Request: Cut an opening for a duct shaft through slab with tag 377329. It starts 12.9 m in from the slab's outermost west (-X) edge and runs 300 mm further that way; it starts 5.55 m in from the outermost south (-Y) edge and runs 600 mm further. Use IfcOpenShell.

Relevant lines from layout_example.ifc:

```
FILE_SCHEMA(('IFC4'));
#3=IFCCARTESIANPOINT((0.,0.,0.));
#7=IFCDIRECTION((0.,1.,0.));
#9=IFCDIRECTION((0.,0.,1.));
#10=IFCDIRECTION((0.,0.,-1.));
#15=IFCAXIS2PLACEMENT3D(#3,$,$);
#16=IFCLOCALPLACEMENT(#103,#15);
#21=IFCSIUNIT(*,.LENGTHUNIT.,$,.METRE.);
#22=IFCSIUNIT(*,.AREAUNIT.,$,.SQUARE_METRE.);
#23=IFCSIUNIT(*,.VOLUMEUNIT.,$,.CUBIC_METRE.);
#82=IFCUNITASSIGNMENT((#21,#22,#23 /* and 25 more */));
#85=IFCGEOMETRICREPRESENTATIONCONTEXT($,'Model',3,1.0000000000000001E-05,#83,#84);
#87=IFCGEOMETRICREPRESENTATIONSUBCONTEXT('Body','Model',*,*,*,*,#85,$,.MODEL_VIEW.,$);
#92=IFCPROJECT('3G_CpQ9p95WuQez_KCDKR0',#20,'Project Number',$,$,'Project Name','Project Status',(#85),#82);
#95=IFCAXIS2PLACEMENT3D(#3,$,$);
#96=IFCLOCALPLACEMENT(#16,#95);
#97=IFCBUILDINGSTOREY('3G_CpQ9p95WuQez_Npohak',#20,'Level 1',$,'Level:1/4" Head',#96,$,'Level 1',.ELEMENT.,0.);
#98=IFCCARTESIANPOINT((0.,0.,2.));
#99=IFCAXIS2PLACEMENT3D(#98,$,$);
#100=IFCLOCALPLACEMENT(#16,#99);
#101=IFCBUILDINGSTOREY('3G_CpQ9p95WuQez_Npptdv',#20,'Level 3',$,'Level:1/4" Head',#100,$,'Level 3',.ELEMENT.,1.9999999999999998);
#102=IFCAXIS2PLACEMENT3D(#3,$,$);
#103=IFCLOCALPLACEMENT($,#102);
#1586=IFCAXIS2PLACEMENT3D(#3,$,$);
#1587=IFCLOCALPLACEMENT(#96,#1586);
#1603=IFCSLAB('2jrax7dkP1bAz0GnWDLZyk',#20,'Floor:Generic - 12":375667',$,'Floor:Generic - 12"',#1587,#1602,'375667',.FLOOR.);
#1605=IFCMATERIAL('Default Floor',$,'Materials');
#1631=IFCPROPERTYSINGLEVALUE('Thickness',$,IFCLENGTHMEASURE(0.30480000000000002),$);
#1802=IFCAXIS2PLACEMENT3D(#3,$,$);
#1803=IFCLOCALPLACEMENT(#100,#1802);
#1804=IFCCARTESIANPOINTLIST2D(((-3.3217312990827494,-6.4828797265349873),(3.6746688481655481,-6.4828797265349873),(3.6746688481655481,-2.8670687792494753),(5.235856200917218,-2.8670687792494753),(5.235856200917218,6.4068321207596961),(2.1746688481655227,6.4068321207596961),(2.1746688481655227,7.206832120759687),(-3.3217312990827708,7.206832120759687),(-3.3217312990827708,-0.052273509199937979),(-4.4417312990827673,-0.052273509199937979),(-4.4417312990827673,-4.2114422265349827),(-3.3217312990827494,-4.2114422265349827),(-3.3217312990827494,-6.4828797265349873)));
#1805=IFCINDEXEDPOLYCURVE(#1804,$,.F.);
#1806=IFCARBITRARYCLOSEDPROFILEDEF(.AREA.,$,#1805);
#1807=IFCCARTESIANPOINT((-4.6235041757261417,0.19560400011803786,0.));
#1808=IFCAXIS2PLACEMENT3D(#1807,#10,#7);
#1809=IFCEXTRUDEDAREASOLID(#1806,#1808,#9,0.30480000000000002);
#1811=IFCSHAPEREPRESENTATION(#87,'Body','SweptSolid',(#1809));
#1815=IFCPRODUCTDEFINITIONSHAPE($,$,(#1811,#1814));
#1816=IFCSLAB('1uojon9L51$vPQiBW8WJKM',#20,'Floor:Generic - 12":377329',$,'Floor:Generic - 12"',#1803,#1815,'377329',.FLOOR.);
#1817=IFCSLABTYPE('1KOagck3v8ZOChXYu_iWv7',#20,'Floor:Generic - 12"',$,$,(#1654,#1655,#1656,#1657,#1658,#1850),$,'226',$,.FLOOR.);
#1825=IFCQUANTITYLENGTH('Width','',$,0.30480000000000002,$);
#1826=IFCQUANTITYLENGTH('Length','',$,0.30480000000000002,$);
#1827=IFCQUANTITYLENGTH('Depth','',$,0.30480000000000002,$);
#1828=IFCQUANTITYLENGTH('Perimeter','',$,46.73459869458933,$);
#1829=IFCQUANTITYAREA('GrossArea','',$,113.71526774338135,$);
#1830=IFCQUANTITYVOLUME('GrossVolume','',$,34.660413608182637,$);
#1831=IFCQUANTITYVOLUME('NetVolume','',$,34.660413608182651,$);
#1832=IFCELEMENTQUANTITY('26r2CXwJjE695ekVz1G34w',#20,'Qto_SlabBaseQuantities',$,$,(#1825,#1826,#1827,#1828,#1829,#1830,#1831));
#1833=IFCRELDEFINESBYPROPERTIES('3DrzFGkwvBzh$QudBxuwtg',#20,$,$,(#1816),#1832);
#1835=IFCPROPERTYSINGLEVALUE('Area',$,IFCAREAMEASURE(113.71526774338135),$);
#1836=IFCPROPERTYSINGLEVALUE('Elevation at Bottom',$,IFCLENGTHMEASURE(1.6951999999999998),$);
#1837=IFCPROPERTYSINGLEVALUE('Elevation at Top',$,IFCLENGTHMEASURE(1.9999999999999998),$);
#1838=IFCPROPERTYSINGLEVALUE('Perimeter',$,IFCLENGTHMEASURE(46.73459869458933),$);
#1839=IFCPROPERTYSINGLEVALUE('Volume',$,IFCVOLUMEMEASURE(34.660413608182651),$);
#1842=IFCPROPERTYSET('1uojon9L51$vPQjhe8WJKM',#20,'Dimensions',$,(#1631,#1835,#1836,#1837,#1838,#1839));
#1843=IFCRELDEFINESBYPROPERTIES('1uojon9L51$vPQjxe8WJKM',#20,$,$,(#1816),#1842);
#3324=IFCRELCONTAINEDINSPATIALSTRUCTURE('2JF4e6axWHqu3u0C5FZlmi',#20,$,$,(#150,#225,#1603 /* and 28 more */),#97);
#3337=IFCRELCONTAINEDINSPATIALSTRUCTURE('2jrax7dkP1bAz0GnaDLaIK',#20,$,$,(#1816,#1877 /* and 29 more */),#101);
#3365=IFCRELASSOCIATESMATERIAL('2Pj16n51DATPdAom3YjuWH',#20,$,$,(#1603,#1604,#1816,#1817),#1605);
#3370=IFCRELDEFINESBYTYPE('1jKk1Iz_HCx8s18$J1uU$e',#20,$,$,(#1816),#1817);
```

```python
import numpy as np
import ifcopenshell
import ifcopenshell.api.feature
import ifcopenshell.api.geometry
import ifcopenshell.api.pset
import ifcopenshell.api.root
import ifcopenshell.geom
import ifcopenshell.util.element
import ifcopenshell.util.placement
import ifcopenshell.util.representation
import ifcopenshell.util.shape
import ifcopenshell.util.unit

model = ifcopenshell.open("layout_example.ifc")
unit_scale = ifcopenshell.util.unit.calculate_unit_scale(model)
area_scale = ifcopenshell.util.unit.calculate_unit_scale(model, "AREAUNIT")
volume_scale = ifcopenshell.util.unit.calculate_unit_scale(model, "VOLUMEUNIT")
settings = ifcopenshell.geom.settings()


def volume(element):
    """Net volume in cubic metres, openings subtracted."""
    shape = ifcopenshell.geom.create_shape(settings, element)
    return ifcopenshell.util.shape.get_volume(shape.geometry)


slab = model.by_guid("1uojon9L51$vPQiBW8WJKM")
before = volume(slab)

# Extent in the slab's own axes, in metres. The edges named are its -X and -Y sides.
slab_shape = ifcopenshell.geom.create_shape(settings, slab)
vertices = ifcopenshell.util.shape.get_vertices(slab_shape.geometry)
x_min, y_min, bottom = vertices.min(axis=0)
top = vertices[:, 2].max()

opening = ifcopenshell.api.root.create_entity(model, ifc_class="IfcOpeningElement", name="Duct shaft opening", predefined_type="OPENING")
context = ifcopenshell.util.representation.get_context(model, "Model", "Body", "MODEL_VIEW")
width, depth = 0.3, 0.6
outline = [(0.0, 0.0), (width, 0.0), (width, depth), (0.0, depth), (0.0, 0.0)]
# Overshoot both faces by 50 mm so the cut is clean.
shape = ifcopenshell.api.geometry.add_slab_representation(
    model, context=context, depth=top - bottom + 0.1, polyline=outline
)
ifcopenshell.api.geometry.assign_representation(model, product=opening, representation=shape)

matrix = ifcopenshell.util.placement.get_local_placement(slab.ObjectPlacement)
matrix[:, 3] = matrix @ np.append(np.array([x_min + 12.9, y_min + 5.55, bottom - 0.05]) / unit_scale, 1.0)
ifcopenshell.api.geometry.edit_object_placement(model, product=opening, matrix=matrix, is_si=False)
ifcopenshell.api.feature.add_feature(model, feature=opening, element=slab)

after = volume(slab)

# Update the slab's stored quantities.
qto = model.by_id(ifcopenshell.util.element.get_pset(slab, "Qto_SlabBaseQuantities", should_inherit=False)["id"])
ifcopenshell.api.pset.edit_qto(model, qto=qto, properties={"NetVolume": after / volume_scale})
pset = model.by_id(ifcopenshell.util.element.get_pset(slab, "Dimensions", should_inherit=False)["id"])
ifcopenshell.api.pset.edit_pset(model, pset=pset, properties={
    "Area": model.create_entity("IfcAreaMeasure", after / (top - bottom) / area_scale),
    "Volume": model.create_entity("IfcVolumeMeasure", after / volume_scale),
})

print(f"slab volume {before:.3f} -> {after:.3f} m3")

model.write("layout_example_edited.ifc")
```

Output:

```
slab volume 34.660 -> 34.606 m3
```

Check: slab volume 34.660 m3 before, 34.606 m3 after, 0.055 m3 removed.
